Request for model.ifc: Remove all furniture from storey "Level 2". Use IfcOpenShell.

First a look at what the model holds.

```python
import ifcopenshell
import ifcopenshell.util.element

model = ifcopenshell.open("model.ifc")
print(model.schema)
storey = next(s for s in model.by_type("IfcBuildingStorey") if s.Name == "Level 2")
furniture = [e for e in ifcopenshell.util.element.get_decomposition(storey) if e.is_a("IfcFurnishingElement")]
seen = {}
for e in furniture:
    element_type = ifcopenshell.util.element.get_type(e)
    name = element_type.Name if element_type not in (None, e) else None
    seen[name] = seen.get(name, 0) + 1
for name, count in sorted(seen.items(), key=str):
    print(count, "x", name)
```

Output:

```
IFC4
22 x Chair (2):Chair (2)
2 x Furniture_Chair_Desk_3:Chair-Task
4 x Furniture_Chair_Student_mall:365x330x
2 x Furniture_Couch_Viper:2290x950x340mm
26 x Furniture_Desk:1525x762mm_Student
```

```python
import ifcopenshell
import ifcopenshell.api.root
import ifcopenshell.util.element

model = ifcopenshell.open("model.ifc")

storey = next(s for s in model.by_type("IfcBuildingStorey") if s.Name == "Level 2")
furniture = [e for e in ifcopenshell.util.element.get_decomposition(storey) if e.is_a("IfcFurnishingElement")]

for e in furniture:
    ifcopenshell.api.root.remove_product(model, product=e)
print(len(furniture), "removed")

model.write("model_v2.ifc")
```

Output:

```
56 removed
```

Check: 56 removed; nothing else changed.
